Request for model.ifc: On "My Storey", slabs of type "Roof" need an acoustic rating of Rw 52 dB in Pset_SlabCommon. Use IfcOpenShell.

First a look at what the model holds.

```python
import ifcopenshell
import ifcopenshell.util.element

model = ifcopenshell.open("model.ifc")
print(model.schema)
storey = next(s for s in model.by_type("IfcBuildingStorey") if s.Name == "My Storey")
slabs = [e for e in ifcopenshell.util.element.get_decomposition(storey) if e.is_a("IfcSlab")]
seen = {}
for e in slabs:
    element_type = ifcopenshell.util.element.get_type(e)
    key = (element_type.Name if element_type != e and element_type else None, ifcopenshell.util.element.get_pset(e, "Pset_SlabCommon", "AcousticRating"))
    seen[key] = seen.get(key, 0) + 1
for (name, value), count in sorted(seen.items(), key=str):
    print(count, "x", name, "|", value)
```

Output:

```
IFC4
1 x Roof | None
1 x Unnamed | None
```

```python
import ifcopenshell
import ifcopenshell.api.pset
import ifcopenshell.util.element

model = ifcopenshell.open("model.ifc")

storey = next(s for s in model.by_type("IfcBuildingStorey") if s.Name == "My Storey")
slabs = [e for e in ifcopenshell.util.element.get_decomposition(storey) if e.is_a("IfcSlab")]

count = 0
for e in slabs:
    element_type = ifcopenshell.util.element.get_type(e)
    if element_type in (None, e) or element_type.Name != "Roof":
        continue
    # add_pset returns the element's existing set when there is one.
    pset = ifcopenshell.api.pset.add_pset(model, product=e, name="Pset_SlabCommon")
    ifcopenshell.api.pset.edit_pset(model, pset=pset, properties={"AcousticRating": "Rw 52 dB"})
    count += 1

print(count, "slabs updated")

model.write("model-out.ifc")
```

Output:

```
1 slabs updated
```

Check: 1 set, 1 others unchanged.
